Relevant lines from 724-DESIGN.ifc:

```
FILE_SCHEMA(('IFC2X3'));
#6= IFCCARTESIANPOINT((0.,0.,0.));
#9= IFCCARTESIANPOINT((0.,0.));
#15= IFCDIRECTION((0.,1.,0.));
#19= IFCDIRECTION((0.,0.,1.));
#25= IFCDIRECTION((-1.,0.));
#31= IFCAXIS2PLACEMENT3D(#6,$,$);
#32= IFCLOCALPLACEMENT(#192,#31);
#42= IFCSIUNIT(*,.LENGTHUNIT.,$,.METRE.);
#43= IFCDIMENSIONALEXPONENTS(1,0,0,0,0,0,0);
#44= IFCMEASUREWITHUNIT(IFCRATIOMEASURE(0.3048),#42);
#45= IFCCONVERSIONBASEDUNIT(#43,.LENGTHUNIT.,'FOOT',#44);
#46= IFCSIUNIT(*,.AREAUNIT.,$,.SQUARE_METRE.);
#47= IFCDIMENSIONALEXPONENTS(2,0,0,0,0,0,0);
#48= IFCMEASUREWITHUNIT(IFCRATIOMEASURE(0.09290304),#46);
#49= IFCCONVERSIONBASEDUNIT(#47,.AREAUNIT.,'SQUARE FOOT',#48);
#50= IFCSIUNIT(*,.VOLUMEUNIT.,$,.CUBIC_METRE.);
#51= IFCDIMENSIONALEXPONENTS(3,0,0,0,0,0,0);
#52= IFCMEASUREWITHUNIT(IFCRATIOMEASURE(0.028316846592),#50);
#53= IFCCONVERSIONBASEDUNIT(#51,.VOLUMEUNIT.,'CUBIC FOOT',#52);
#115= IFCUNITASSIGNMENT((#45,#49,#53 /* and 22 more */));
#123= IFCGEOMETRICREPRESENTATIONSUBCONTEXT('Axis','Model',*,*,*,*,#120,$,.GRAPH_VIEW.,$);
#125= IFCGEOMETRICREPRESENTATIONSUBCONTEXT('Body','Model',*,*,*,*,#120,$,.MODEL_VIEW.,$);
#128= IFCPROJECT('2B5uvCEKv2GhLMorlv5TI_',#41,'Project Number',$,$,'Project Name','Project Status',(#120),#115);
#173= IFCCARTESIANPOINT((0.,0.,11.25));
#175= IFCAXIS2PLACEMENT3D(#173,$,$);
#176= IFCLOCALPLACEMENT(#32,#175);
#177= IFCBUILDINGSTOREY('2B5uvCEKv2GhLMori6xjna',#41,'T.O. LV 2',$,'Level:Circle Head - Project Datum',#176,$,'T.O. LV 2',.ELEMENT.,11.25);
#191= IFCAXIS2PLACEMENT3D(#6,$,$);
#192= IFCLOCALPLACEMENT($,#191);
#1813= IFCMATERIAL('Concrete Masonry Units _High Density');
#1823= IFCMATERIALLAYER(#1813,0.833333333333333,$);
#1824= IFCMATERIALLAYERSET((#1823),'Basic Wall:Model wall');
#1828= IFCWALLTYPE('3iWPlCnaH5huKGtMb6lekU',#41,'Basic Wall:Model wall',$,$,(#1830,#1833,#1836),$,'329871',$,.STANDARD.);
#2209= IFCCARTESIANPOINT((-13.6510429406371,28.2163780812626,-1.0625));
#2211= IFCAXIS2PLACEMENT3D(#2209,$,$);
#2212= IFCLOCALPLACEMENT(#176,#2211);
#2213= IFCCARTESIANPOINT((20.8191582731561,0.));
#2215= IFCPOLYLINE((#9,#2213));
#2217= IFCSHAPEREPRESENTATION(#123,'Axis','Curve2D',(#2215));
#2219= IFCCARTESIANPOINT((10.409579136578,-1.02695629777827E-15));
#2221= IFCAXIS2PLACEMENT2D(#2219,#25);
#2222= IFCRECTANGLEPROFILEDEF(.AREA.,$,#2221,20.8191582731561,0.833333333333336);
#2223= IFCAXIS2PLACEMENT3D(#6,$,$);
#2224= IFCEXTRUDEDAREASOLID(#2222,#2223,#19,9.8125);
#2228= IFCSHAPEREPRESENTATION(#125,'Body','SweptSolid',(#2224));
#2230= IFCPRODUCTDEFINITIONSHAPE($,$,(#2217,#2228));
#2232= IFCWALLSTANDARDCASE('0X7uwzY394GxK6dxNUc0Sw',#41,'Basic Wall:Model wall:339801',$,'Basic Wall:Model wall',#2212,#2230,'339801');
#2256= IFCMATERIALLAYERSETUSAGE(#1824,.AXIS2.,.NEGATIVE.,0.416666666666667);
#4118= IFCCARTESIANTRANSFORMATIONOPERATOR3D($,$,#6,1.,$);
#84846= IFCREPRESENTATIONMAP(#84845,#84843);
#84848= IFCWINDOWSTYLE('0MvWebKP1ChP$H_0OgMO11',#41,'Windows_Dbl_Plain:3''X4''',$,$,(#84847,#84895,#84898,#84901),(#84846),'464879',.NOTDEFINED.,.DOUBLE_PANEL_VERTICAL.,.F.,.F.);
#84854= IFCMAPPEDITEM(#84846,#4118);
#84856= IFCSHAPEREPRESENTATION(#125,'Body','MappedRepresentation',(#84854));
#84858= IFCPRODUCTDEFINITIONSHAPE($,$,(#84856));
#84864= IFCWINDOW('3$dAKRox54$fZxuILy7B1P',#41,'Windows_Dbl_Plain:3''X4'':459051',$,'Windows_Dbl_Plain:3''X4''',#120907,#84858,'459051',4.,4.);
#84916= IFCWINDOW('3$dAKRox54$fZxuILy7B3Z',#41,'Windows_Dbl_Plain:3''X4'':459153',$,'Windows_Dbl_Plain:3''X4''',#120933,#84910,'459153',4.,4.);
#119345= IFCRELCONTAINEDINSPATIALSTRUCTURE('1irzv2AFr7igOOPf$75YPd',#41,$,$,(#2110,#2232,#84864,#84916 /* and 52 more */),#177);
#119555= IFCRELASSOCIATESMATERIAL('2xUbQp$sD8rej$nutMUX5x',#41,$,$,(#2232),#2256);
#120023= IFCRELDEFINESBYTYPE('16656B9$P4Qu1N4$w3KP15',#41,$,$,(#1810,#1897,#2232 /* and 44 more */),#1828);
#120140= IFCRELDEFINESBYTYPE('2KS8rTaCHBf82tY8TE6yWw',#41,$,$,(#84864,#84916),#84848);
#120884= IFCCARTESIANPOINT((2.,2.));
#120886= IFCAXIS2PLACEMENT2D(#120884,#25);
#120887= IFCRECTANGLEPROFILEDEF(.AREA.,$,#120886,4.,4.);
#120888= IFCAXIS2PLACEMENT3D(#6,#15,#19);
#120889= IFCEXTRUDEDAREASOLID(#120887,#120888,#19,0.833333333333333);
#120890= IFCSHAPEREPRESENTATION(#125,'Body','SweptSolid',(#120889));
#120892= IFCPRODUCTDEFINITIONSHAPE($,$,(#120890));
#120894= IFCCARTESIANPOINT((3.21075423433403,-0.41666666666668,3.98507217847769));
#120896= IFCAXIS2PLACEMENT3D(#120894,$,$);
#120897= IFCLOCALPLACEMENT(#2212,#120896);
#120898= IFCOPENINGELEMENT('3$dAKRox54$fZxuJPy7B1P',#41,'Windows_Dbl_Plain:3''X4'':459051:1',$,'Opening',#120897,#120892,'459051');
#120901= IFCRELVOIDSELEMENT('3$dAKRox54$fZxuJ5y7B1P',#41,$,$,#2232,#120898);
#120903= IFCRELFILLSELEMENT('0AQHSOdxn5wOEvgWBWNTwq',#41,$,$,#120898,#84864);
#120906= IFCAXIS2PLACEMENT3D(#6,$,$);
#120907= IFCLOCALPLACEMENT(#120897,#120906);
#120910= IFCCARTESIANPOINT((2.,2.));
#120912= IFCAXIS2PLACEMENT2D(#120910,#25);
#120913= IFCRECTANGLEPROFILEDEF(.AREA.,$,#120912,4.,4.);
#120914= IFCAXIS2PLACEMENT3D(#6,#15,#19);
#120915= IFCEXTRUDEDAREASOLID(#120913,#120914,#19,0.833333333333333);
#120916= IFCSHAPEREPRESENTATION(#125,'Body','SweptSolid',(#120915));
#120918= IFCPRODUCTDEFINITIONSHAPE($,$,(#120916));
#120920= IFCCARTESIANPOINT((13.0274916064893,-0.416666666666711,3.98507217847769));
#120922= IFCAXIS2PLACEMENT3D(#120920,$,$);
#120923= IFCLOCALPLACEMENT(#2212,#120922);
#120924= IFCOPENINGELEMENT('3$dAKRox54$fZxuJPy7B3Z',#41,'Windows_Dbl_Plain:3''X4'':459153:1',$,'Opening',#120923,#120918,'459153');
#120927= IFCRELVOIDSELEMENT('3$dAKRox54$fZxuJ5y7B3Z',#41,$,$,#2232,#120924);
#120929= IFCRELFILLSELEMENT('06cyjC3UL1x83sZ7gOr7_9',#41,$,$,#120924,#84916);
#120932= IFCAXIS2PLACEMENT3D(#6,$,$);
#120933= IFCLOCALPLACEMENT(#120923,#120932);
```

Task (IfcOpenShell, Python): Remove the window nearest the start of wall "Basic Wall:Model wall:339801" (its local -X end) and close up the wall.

```python
import ifcopenshell
import ifcopenshell.api.feature
import ifcopenshell.api.root
import ifcopenshell.geom
import ifcopenshell.util.shape

model = ifcopenshell.open("724-DESIGN.ifc")
settings = ifcopenshell.geom.settings()


def volume(element):
    """Net volume in cubic metres, openings subtracted."""
    shape = ifcopenshell.geom.create_shape(settings, element)
    return ifcopenshell.util.shape.get_volume(shape.geometry)


window = model.by_id(84864)
opening = window.FillsVoids[0].RelatingOpeningElement
wall = opening.VoidsElements[0].RelatingBuildingElement
before = volume(wall)

ifcopenshell.api.root.remove_product(model, product=window)
ifcopenshell.api.feature.remove_feature(model, feature=opening)

after = volume(wall)

print(f"wall volume {before:.3f} -> {after:.3f} m3")

model.write("724-DESIGN_rev.ifc")
```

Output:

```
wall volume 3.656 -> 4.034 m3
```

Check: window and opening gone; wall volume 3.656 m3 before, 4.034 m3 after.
